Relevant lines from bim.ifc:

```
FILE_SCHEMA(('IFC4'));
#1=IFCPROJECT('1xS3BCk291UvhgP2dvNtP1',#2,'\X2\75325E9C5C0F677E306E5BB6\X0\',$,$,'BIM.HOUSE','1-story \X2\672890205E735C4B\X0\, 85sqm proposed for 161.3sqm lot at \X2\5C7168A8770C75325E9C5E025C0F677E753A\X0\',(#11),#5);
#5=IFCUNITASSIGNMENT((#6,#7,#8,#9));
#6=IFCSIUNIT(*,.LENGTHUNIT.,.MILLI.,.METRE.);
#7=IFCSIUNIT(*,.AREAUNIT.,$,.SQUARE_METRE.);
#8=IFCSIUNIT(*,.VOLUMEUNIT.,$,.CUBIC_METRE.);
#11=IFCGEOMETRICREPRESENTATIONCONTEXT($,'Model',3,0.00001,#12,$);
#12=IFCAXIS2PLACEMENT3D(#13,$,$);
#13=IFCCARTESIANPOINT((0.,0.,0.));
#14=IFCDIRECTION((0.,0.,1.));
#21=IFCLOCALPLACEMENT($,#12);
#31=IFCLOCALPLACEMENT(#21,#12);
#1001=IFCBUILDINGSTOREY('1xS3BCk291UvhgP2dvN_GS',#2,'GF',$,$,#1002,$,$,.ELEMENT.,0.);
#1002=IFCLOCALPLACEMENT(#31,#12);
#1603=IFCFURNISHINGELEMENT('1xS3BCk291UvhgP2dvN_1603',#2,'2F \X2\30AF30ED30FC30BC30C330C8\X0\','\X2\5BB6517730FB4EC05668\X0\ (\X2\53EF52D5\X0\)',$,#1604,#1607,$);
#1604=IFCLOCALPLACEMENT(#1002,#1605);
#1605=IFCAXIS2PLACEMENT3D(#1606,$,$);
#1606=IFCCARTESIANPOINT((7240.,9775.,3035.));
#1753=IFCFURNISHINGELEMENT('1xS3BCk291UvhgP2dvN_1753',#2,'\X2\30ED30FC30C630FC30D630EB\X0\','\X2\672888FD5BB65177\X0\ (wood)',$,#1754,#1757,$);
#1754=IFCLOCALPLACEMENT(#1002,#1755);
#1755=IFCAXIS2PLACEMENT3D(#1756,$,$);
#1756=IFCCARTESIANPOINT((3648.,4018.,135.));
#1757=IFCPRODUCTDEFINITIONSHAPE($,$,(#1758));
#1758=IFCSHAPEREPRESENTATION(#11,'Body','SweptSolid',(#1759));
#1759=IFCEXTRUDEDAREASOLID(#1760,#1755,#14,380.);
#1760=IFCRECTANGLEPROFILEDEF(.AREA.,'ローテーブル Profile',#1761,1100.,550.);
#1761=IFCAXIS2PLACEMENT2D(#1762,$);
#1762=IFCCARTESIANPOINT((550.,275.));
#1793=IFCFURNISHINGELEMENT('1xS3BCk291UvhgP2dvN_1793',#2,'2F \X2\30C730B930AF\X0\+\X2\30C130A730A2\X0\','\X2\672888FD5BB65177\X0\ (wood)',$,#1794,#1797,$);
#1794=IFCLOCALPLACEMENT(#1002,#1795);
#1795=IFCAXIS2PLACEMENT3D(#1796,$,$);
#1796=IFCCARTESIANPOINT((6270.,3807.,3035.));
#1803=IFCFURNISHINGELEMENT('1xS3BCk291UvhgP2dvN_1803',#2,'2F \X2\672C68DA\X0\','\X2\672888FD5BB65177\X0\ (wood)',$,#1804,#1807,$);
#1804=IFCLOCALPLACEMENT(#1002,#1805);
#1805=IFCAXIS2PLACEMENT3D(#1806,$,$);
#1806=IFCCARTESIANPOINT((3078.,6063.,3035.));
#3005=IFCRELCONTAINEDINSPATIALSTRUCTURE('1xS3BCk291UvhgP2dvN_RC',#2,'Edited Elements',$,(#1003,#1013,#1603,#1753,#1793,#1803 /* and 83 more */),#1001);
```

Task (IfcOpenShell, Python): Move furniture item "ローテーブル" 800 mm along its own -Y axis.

```python
import ifcopenshell
import ifcopenshell.api.geometry
import ifcopenshell.util.placement
import ifcopenshell.util.unit

model = ifcopenshell.open("bim.ifc")
unit_scale = ifcopenshell.util.unit.calculate_unit_scale(model)

item = model.by_guid("1xS3BCk291UvhgP2dvN_1753")
matrix = ifcopenshell.util.placement.get_local_placement(item.ObjectPlacement)
matrix[:3, 3] -= matrix[:3, 1] * 0.8 / unit_scale
ifcopenshell.api.geometry.edit_object_placement(model, product=item, matrix=matrix, is_si=False)

print(ifcopenshell.util.placement.get_local_placement(item.ObjectPlacement).round(3) + 0.0)

model.write("bim_v2.ifc")
```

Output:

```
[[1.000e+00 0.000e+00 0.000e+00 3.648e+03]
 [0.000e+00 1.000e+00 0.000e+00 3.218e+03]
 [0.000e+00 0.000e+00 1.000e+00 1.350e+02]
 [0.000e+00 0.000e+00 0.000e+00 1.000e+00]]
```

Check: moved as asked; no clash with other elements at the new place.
